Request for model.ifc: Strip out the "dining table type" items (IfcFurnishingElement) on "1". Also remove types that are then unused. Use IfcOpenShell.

First a look at what the model holds.

```python
import ifcopenshell
import ifcopenshell.util.element

model = ifcopenshell.open("model.ifc")
print(model.schema)
storey = next(s for s in model.by_type("IfcBuildingStorey") if s.Name == "1")
furniture = [e for e in ifcopenshell.util.element.get_decomposition(storey) if e.is_a("IfcFurnishingElement")]
seen = {}
for e in furniture:
    element_type = ifcopenshell.util.element.get_type(e)
    name = element_type.Name if element_type not in (None, e) else None
    seen[name] = seen.get(name, 0) + 1
for name, count in sorted(seen.items(), key=str):
    print(count, "x", name)
```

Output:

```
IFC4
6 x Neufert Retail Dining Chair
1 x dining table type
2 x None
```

```python
import ifcopenshell
import ifcopenshell.api.root
import ifcopenshell.util.element

model = ifcopenshell.open("model.ifc")

storey = next(s for s in model.by_type("IfcBuildingStorey") if s.Name == "1")
furniture = [e for e in ifcopenshell.util.element.get_decomposition(storey) if e.is_a("IfcFurnishingElement")]
targets = [e for e in furniture if (t := ifcopenshell.util.element.get_type(e)) not in (None, e) and t.Name == "dining table type"]
types = {ifcopenshell.util.element.get_type(e) for e in targets} - {None, *targets}

for e in targets:
    ifcopenshell.api.root.remove_product(model, product=e)
print(len(targets), "removed")

unused = [t for t in types if not ifcopenshell.util.element.get_types(t)]
for t in unused:
    ifcopenshell.api.root.remove_product(model, product=t)
print(len(unused), "unused types removed")

model.write("model_rev.ifc")
```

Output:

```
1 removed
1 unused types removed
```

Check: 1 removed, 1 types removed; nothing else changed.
